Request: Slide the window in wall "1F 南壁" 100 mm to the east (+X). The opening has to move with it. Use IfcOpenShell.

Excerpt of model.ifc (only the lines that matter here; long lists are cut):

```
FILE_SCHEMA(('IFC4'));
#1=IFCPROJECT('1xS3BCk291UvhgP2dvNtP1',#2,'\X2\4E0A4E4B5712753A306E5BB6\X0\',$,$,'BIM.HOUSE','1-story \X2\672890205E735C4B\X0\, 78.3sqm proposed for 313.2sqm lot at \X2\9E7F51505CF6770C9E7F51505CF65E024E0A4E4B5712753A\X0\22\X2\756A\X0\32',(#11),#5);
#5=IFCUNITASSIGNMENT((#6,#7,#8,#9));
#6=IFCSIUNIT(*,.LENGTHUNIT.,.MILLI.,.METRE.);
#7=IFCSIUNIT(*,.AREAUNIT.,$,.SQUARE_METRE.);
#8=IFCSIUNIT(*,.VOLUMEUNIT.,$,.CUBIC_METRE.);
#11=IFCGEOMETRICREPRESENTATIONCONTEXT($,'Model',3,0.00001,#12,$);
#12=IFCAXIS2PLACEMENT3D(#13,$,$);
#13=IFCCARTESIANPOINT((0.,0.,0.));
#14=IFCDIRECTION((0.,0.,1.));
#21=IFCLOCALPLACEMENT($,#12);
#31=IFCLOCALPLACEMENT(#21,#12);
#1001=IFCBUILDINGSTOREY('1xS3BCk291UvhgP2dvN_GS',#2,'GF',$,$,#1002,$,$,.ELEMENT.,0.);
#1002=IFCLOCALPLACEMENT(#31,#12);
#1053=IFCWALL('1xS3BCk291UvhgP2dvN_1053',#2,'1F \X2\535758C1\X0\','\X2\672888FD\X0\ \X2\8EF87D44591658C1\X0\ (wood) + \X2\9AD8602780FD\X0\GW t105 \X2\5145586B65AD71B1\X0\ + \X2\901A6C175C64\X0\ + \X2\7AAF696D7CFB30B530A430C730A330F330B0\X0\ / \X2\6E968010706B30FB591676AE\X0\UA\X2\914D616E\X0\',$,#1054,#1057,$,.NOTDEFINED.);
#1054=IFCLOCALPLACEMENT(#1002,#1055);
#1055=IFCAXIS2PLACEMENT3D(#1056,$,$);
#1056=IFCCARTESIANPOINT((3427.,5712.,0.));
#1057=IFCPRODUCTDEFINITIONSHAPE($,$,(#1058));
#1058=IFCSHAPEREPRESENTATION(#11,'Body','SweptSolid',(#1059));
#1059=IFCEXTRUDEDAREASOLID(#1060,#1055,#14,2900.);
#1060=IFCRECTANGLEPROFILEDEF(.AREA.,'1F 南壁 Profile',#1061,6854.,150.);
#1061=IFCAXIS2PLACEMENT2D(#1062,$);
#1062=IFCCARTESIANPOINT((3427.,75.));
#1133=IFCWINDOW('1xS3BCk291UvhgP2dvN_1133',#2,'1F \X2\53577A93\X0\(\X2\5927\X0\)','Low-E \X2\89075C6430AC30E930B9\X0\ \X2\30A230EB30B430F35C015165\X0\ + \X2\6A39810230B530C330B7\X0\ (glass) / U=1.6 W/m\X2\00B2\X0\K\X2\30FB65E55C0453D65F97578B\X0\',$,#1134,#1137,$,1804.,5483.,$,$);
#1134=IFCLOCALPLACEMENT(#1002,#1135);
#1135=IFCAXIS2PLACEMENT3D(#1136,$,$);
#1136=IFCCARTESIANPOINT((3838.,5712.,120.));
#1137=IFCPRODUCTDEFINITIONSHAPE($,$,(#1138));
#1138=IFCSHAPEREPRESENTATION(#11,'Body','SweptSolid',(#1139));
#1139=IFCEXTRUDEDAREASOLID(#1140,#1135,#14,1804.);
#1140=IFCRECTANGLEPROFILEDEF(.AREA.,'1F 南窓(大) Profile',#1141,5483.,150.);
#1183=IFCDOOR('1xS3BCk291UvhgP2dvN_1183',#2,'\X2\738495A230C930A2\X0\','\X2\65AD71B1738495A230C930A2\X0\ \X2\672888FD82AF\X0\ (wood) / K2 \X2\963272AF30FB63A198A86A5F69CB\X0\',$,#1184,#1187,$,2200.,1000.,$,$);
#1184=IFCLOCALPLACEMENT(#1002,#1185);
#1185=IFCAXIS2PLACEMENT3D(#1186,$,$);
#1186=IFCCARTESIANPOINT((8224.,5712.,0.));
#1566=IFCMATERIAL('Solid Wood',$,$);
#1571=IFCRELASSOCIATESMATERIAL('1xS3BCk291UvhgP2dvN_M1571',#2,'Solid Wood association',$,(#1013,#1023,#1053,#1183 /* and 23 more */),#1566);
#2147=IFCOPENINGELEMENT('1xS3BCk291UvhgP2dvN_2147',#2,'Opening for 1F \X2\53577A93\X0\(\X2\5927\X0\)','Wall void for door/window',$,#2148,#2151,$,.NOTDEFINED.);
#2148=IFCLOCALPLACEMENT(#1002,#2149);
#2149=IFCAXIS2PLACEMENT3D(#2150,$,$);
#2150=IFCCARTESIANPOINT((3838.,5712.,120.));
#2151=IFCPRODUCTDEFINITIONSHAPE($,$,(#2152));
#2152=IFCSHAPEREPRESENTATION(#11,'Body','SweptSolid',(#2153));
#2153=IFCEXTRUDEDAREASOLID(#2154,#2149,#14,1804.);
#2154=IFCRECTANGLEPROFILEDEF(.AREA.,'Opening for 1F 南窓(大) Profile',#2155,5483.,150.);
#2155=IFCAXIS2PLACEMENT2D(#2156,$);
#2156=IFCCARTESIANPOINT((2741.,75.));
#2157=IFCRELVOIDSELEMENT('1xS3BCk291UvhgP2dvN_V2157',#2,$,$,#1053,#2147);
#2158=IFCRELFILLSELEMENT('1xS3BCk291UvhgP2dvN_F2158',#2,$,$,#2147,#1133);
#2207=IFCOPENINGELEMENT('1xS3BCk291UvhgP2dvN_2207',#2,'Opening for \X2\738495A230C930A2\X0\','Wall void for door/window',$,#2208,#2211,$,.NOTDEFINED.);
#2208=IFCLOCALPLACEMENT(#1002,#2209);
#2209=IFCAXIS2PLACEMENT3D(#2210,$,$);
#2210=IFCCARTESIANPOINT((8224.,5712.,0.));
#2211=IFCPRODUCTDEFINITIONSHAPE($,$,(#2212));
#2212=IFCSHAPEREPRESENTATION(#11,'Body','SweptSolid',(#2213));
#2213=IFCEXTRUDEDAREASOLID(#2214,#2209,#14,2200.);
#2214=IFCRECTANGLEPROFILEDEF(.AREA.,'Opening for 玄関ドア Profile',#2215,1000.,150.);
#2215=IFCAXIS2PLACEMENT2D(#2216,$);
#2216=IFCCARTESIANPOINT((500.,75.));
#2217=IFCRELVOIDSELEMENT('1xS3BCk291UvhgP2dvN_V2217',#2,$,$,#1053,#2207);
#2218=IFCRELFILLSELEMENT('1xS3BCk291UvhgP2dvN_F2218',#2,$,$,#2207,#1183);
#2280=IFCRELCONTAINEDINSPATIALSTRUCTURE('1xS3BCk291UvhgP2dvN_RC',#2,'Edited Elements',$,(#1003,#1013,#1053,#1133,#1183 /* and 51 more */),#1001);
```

```python
import ifcopenshell
import ifcopenshell.api.geometry
import ifcopenshell.util.placement
import ifcopenshell.util.unit

model = ifcopenshell.open("model.ifc")
unit_scale = ifcopenshell.util.unit.calculate_unit_scale(model)

window = model.by_guid("1xS3BCk291UvhgP2dvN_1133")
opening = window.FillsVoids[0].RelatingOpeningElement
wall = opening.VoidsElements[0].RelatingBuildingElement

wall_matrix = ifcopenshell.util.placement.get_local_placement(wall.ObjectPlacement)
shift = wall_matrix[:3, 0] * 0.1 / unit_scale
before = ifcopenshell.util.placement.get_local_placement(window.ObjectPlacement)[:3, 3].copy()

# The window is not placed relative to its opening, so move both.
for product in (opening, window):
    matrix = ifcopenshell.util.placement.get_local_placement(product.ObjectPlacement)
    matrix[:3, 3] += shift
    ifcopenshell.api.geometry.edit_object_placement(model, product=product, matrix=matrix, is_si=False)

after = ifcopenshell.util.placement.get_local_placement(window.ObjectPlacement)[:3, 3]
print("window moved by", (after - before).round(3) + 0.0)

model.write("model_edited.ifc")
```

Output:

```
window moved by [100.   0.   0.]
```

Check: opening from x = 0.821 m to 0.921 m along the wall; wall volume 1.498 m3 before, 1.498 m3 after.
